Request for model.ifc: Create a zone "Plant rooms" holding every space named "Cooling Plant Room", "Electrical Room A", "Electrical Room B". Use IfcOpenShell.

First a look at what the model holds.

```python
import ifcopenshell

model = ifcopenshell.open("model.ifc")
print(model.schema)
seen = {}
for space in model.by_type("IfcSpace"):
    seen[space.LongName] = seen.get(space.LongName, 0) + 1
for name, count in sorted(seen.items(), key=str):
    print(count, "x", name)
print("zones:", [z.Name for z in model.by_type("IfcZone")][:20])
```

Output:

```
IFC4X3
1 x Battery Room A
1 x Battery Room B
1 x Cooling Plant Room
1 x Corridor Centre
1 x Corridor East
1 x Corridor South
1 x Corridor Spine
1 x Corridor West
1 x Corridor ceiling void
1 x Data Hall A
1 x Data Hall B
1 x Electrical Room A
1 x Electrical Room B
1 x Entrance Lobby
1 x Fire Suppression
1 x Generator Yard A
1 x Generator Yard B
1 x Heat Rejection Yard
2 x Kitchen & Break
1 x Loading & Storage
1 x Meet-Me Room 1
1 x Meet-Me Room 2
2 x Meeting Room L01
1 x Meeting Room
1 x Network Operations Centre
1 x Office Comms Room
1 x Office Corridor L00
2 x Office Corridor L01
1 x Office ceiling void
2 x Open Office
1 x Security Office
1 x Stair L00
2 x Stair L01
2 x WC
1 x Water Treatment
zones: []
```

```python
import ifcopenshell
import ifcopenshell.api.group
import ifcopenshell.api.root

model = ifcopenshell.open("model.ifc")

names = {"Cooling Plant Room", "Electrical Room A", "Electrical Room B"}
spaces = [s for s in model.by_type("IfcSpace") if s.LongName in names]

zone = ifcopenshell.api.root.create_entity(model, ifc_class="IfcZone", name="Plant rooms")
ifcopenshell.api.group.assign_group(model, products=spaces, group=zone)
print(len(spaces), "spaces in", zone.Name)

model.write("model_edited.ifc")
```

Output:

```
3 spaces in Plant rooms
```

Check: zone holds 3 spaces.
